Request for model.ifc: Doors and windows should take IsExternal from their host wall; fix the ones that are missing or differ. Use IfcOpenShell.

First a look at what the model holds.

```python
import ifcopenshell
import ifcopenshell.util.element

model = ifcopenshell.open("model.ifc")
print(model.schema)
seen = {}
for e in model.by_type("IfcDoor") + model.by_type("IfcWindow"):
    if not e.FillsVoids:
        continue
    host = e.FillsVoids[0].RelatingOpeningElement.VoidsElements[0].RelatingBuildingElement
    own = ifcopenshell.util.element.get_pset(e, f"Pset_{e.is_a()[3:].removesuffix('StandardCase')}Common", "IsExternal")
    wall = ifcopenshell.util.element.get_pset(host, "Pset_WallCommon", "IsExternal")
    seen[e.is_a(), own, wall] = seen.get((e.is_a(), own, wall), 0) + 1
for (cls, own, wall), count in sorted(seen.items(), key=str):
    print(count, cls, "IsExternal:", own, "| host wall:", wall)
```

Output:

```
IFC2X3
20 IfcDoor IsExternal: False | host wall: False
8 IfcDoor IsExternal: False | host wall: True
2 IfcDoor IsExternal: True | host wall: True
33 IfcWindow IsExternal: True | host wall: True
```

```python
import ifcopenshell
import ifcopenshell.api.pset
import ifcopenshell.util.element

model = ifcopenshell.open("model.ifc")

count = 0
for ifc_class, pset_name in (("IfcDoor", "Pset_DoorCommon"), ("IfcWindow", "Pset_WindowCommon")):
    for e in model.by_type(ifc_class):
        if not e.FillsVoids:
            continue
        host = e.FillsVoids[0].RelatingOpeningElement.VoidsElements[0].RelatingBuildingElement
        external = ifcopenshell.util.element.get_pset(host, "Pset_WallCommon", "IsExternal")
        if external is None or ifcopenshell.util.element.get_pset(e, pset_name, "IsExternal") == external:
            continue
        pset = ifcopenshell.api.pset.add_pset(model, product=e, name=pset_name)
        ifcopenshell.api.pset.edit_pset(model, pset=pset, properties={"IsExternal": external})
        count += 1

print(count, "updated")

model.write("model_rev.ifc")
```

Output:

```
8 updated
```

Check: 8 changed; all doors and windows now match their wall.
